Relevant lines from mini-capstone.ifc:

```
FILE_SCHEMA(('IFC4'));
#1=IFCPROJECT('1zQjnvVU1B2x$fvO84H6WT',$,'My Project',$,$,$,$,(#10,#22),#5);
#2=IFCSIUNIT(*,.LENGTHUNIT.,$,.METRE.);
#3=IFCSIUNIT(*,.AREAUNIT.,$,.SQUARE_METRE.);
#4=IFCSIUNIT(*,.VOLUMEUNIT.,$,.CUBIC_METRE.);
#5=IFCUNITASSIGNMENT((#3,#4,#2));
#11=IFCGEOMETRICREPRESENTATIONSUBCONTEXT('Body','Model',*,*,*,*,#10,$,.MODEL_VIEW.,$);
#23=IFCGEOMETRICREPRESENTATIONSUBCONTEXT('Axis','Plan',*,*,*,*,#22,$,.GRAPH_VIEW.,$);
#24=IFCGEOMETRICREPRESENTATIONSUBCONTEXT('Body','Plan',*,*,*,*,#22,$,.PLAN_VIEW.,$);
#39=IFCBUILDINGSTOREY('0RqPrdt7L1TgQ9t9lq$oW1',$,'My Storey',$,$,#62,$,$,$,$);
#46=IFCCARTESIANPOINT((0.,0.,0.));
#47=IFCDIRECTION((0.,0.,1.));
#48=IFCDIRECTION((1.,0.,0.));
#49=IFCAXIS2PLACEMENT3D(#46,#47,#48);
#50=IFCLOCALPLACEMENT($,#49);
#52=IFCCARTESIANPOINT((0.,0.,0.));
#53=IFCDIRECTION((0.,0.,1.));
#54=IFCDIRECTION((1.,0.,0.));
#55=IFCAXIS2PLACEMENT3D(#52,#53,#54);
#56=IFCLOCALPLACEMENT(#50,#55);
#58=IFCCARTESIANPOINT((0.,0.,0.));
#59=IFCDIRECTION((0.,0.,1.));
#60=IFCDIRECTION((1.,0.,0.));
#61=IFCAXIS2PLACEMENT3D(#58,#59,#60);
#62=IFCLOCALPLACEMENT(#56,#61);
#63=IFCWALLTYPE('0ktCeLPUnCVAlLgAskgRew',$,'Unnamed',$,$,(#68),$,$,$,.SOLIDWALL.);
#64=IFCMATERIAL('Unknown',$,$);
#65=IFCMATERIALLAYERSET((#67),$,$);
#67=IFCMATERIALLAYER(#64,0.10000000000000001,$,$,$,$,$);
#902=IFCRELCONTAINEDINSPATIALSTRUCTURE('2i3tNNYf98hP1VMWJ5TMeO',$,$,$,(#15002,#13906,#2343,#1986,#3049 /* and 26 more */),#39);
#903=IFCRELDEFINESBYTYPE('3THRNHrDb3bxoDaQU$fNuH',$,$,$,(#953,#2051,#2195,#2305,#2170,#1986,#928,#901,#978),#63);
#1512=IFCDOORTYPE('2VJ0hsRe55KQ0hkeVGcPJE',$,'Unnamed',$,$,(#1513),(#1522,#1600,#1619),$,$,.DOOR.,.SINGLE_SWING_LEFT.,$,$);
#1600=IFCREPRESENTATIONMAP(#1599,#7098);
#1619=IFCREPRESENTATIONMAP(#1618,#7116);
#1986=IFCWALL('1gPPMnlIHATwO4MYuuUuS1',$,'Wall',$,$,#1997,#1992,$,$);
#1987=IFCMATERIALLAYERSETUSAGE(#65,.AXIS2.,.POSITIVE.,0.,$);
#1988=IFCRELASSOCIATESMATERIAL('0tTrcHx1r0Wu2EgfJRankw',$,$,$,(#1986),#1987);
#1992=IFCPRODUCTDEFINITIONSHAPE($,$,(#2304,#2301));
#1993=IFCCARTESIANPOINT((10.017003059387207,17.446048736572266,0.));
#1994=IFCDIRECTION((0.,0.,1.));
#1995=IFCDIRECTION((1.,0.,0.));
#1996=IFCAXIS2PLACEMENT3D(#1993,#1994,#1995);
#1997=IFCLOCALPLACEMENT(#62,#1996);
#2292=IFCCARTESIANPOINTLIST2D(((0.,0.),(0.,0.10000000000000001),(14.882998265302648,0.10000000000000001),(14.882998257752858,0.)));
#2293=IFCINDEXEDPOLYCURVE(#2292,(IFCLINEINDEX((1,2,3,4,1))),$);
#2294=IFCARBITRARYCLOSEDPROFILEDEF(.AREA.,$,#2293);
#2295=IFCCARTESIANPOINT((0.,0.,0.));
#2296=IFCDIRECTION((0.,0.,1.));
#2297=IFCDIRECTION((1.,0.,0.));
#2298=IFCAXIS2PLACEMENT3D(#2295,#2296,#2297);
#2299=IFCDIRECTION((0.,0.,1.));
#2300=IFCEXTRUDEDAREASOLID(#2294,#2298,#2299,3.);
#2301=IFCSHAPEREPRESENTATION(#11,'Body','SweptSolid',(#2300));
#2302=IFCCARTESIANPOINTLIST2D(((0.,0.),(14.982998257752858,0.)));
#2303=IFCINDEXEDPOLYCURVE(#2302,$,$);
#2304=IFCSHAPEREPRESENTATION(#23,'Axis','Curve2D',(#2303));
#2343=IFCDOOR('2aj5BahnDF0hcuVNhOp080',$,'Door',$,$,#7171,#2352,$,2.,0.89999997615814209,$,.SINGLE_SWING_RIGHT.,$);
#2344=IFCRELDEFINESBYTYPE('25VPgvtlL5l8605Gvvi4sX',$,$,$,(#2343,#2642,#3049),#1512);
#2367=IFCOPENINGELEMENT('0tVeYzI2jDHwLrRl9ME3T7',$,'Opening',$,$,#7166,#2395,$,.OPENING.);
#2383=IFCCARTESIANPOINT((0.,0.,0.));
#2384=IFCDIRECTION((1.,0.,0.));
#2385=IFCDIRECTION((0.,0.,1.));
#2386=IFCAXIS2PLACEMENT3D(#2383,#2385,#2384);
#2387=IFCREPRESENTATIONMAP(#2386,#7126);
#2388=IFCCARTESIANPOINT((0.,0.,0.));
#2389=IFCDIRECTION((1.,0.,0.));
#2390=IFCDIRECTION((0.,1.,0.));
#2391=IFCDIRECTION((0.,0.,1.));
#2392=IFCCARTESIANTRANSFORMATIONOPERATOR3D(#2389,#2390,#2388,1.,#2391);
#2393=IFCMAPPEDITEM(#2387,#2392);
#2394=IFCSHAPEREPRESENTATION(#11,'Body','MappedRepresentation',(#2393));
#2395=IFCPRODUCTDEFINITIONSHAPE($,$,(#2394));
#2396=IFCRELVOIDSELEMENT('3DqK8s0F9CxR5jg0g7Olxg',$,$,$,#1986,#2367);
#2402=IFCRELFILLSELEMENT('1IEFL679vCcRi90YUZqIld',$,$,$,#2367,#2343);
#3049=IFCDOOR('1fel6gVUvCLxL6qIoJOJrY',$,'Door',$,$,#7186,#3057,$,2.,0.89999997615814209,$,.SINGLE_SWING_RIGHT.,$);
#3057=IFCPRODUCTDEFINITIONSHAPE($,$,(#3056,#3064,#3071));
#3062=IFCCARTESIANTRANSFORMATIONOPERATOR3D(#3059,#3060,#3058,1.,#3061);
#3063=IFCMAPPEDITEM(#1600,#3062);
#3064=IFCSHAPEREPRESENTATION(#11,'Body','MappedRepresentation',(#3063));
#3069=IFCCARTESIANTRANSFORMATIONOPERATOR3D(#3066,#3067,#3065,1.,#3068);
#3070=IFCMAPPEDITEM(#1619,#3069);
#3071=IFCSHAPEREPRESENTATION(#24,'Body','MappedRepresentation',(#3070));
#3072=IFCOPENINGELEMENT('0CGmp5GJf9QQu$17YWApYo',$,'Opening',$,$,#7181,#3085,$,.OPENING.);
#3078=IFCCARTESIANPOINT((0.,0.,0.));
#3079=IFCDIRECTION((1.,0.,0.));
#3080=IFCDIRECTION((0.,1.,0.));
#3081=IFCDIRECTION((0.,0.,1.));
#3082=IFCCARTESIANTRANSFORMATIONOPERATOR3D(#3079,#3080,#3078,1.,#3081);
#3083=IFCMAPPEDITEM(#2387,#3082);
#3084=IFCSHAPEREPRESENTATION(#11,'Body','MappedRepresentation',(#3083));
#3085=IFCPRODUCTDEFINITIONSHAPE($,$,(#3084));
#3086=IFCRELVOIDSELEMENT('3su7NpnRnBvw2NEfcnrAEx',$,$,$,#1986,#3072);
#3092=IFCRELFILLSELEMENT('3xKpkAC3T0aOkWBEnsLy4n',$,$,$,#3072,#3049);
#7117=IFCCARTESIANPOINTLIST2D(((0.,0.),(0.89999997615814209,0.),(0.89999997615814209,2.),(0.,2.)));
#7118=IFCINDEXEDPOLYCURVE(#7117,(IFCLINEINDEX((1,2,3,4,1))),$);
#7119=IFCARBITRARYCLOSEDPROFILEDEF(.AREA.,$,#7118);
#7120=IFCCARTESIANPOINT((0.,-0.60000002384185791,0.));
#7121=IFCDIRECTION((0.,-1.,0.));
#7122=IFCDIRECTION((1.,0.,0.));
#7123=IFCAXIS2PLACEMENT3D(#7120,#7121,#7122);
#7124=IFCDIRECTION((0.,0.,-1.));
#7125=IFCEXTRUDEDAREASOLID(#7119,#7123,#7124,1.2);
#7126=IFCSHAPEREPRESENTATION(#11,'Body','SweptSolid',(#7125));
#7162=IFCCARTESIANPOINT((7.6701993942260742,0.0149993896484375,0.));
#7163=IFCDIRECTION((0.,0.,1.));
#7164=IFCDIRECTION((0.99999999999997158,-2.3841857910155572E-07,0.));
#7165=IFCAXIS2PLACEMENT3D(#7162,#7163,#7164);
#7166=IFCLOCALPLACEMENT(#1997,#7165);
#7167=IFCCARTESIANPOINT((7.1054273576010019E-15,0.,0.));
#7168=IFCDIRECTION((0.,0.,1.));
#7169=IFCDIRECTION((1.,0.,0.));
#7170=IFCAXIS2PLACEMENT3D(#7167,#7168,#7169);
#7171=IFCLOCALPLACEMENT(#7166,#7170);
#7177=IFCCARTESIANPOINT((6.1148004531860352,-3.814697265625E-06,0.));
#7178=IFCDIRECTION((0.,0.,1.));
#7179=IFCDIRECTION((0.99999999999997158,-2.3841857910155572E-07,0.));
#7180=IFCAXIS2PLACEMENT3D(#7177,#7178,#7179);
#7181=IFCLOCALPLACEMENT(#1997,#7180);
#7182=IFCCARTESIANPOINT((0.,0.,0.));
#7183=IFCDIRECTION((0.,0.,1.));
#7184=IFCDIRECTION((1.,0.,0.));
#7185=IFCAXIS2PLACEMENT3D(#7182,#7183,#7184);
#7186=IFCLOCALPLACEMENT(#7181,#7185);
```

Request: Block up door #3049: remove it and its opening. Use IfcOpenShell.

```python
import ifcopenshell
import ifcopenshell.api.feature
import ifcopenshell.api.root
import ifcopenshell.geom
import ifcopenshell.util.shape

model = ifcopenshell.open("mini-capstone.ifc")
settings = ifcopenshell.geom.settings()


def volume(element):
    """Net volume in cubic metres, openings subtracted."""
    shape = ifcopenshell.geom.create_shape(settings, element)
    return ifcopenshell.util.shape.get_volume(shape.geometry)


door = model.by_id(3049)
opening = door.FillsVoids[0].RelatingOpeningElement
wall = opening.VoidsElements[0].RelatingBuildingElement
before = volume(wall)

ifcopenshell.api.root.remove_product(model, product=door)
ifcopenshell.api.feature.remove_feature(model, feature=opening)

after = volume(wall)

print(f"wall volume {before:.3f} -> {after:.3f} m3")

model.write("mini-capstone_edited.ifc")
```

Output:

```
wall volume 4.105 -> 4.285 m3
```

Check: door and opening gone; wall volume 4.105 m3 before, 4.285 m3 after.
